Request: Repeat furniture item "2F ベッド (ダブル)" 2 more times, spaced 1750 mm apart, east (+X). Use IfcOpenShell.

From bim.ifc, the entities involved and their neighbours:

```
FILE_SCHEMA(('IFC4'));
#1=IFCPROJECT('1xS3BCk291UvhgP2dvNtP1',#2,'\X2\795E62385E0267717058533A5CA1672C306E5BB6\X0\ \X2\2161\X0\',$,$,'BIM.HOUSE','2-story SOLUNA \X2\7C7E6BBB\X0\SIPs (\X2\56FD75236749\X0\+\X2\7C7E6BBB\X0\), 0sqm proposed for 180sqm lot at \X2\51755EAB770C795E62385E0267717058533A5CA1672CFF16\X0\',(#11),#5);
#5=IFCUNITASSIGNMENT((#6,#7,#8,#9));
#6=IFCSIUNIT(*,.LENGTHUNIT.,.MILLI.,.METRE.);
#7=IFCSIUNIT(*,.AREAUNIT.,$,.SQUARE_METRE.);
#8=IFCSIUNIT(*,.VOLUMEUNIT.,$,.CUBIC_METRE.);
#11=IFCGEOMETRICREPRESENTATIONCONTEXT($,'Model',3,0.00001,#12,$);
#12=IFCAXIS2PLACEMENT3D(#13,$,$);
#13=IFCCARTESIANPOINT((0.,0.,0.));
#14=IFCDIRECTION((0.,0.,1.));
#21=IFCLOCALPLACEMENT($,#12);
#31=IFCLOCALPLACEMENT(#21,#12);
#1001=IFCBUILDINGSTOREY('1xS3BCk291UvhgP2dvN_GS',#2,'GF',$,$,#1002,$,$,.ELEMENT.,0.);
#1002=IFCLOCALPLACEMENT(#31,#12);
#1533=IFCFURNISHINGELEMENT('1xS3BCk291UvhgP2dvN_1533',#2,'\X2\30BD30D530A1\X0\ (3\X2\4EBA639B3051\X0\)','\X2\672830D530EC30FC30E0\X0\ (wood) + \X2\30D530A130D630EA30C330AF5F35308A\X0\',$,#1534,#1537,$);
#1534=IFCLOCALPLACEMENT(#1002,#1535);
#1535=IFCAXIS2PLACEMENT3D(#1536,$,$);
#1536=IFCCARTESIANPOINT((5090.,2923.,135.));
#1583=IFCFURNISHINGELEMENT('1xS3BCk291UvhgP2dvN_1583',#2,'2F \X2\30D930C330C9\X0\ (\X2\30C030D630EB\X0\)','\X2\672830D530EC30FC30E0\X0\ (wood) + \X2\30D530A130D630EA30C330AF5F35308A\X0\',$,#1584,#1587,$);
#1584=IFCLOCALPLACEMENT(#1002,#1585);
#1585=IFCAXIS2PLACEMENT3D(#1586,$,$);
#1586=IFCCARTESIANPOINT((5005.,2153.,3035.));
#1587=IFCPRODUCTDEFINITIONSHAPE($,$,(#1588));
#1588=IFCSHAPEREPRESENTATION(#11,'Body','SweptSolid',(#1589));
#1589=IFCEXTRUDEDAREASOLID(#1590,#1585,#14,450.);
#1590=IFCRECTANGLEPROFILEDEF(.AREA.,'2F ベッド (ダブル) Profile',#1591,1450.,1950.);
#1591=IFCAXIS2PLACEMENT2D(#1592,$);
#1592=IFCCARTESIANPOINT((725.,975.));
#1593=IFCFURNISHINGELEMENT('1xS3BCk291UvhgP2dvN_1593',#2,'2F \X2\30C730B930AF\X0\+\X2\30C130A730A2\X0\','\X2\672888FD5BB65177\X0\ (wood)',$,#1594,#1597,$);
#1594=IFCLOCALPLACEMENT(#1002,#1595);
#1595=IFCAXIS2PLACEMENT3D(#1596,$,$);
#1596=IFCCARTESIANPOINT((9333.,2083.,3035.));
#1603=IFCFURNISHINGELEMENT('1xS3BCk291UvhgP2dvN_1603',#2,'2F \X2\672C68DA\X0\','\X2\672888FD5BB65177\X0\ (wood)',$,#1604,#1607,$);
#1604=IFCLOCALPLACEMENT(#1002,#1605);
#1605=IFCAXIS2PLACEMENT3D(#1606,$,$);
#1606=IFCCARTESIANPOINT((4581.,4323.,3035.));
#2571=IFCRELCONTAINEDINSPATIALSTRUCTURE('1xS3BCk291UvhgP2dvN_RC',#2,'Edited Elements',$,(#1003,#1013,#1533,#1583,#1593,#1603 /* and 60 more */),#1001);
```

```python
import numpy as np
import ifcopenshell
import ifcopenshell.api.geometry
import ifcopenshell.api.root
import ifcopenshell.util.element
import ifcopenshell.util.placement

model = ifcopenshell.open("bim.ifc")


def reuse_history(source, copy):
    """copy_class also copies each property set's owner history, people and application; keep the originals."""
    for rel in copy.IsDefinedBy:
        if rel.is_a("IfcRelDefinesByProperties") and (history := rel.RelatingPropertyDefinition.OwnerHistory):
            rel.RelatingPropertyDefinition.OwnerHistory = source.OwnerHistory
            ifcopenshell.util.element.remove_deep2(model, history)


source = model.by_id(1583)
base = ifcopenshell.util.placement.get_local_placement(source.ObjectPlacement)
step = np.array([1.0, 0.0, 0.0]) * 1750.0

for i in range(1, 3):
    copy = ifcopenshell.api.root.copy_class(model, product=source)
    copy.Representation = ifcopenshell.util.element.copy_deep(
        model, source.Representation, exclude=["IfcGeometricRepresentationContext", "IfcRepresentationMap"]
    )
    reuse_history(source, copy)
    matrix = base.copy()
    matrix[:3, 3] += i * step
    print("added at", matrix[:3, 3].round(3) + 0.0)
    ifcopenshell.api.geometry.edit_object_placement(model, product=copy, matrix=matrix, is_si=False)

model.write("bim_rev.ifc")
```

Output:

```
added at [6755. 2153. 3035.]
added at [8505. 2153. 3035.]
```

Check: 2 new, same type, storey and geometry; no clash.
